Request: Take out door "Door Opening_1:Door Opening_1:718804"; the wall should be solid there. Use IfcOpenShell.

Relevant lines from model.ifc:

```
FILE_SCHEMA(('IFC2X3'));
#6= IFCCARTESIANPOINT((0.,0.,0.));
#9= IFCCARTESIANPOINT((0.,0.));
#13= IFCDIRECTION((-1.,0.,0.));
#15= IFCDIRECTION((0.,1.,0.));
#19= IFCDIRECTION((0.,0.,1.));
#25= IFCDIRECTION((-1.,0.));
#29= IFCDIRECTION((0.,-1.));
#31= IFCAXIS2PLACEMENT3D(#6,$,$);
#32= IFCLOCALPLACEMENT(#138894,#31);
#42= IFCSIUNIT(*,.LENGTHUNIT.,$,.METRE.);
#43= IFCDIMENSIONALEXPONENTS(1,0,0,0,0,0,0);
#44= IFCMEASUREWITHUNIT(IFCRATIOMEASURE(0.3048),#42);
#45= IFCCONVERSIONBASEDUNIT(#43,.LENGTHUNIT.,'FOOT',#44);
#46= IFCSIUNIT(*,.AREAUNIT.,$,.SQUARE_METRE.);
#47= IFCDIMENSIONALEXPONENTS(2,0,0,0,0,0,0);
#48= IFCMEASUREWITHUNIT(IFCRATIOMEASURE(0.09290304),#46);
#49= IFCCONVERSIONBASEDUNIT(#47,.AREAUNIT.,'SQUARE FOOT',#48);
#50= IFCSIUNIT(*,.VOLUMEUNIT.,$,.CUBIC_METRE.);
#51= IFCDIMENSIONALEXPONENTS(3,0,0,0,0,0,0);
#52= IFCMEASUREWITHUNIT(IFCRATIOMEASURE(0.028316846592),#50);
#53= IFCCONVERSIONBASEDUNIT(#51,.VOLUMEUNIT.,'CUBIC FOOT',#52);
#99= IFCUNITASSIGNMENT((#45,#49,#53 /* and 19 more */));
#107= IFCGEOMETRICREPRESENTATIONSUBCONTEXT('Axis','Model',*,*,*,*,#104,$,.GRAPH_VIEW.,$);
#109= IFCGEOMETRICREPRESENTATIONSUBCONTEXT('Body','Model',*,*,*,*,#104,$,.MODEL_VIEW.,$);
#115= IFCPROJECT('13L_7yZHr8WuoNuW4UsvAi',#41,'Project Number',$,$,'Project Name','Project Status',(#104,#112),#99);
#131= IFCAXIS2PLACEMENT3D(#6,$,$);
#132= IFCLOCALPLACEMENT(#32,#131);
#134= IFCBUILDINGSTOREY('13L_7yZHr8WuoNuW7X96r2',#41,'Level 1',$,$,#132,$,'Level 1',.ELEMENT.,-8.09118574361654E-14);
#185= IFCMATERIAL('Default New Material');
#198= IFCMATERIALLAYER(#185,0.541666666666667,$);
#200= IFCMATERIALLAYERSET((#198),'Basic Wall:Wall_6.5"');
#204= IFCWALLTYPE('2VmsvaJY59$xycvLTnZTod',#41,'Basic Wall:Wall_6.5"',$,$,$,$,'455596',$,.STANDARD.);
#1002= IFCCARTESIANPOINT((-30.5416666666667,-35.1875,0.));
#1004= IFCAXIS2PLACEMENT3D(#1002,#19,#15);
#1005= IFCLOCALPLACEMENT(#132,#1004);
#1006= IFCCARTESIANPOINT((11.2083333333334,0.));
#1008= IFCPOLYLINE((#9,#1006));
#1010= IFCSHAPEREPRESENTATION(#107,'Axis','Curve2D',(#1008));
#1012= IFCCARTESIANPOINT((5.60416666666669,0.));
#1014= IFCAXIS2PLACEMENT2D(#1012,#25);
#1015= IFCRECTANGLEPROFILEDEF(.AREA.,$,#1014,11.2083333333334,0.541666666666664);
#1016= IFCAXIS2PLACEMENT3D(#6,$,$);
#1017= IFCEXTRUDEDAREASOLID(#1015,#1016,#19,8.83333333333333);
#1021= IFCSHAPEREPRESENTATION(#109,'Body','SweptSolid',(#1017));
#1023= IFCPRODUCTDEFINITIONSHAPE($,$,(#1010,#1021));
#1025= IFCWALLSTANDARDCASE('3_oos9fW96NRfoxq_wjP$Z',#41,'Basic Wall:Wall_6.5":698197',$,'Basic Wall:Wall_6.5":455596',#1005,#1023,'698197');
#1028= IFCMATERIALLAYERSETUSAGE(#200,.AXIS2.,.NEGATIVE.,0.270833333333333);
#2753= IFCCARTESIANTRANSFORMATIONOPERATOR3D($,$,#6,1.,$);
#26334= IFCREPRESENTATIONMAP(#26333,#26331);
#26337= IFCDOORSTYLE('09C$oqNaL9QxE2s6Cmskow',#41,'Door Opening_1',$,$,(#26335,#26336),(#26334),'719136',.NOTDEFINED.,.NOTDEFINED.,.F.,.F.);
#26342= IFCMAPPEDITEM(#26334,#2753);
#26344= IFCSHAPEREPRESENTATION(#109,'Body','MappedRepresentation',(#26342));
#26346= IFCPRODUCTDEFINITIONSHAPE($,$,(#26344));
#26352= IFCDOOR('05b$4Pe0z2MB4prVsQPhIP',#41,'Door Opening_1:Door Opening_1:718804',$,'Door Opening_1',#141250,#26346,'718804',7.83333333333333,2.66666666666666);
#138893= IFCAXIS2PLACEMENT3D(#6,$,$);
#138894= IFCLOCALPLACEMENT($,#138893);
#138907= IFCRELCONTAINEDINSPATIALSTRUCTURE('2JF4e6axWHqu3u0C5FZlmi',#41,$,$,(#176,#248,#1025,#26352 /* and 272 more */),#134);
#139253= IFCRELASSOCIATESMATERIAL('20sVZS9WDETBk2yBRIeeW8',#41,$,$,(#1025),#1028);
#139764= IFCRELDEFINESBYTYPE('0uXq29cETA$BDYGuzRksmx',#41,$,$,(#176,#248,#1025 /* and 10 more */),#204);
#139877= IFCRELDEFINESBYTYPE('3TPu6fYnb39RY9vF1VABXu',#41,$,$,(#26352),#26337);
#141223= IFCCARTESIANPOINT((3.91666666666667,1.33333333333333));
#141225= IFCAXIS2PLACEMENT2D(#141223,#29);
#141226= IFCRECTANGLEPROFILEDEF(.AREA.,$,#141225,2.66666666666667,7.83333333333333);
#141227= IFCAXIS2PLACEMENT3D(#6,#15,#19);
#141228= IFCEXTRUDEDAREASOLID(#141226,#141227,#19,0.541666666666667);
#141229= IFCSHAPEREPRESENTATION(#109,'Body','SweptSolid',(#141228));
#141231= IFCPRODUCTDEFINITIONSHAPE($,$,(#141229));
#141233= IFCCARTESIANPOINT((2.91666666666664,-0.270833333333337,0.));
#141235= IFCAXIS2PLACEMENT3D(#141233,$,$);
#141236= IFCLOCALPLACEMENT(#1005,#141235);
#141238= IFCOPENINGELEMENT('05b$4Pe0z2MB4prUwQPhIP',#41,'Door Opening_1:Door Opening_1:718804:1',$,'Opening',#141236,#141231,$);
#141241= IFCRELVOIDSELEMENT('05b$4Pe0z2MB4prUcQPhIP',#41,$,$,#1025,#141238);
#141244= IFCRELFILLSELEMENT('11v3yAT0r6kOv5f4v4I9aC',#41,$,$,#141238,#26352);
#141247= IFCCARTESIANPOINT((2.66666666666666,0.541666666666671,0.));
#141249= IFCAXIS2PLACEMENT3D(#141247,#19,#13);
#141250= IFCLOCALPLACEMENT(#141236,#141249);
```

```python
import ifcopenshell
import ifcopenshell.api.feature
import ifcopenshell.api.root
import ifcopenshell.geom
import ifcopenshell.util.shape

model = ifcopenshell.open("model.ifc")
settings = ifcopenshell.geom.settings()


def volume(element):
    """Net volume in cubic metres, openings subtracted."""
    shape = ifcopenshell.geom.create_shape(settings, element)
    return ifcopenshell.util.shape.get_volume(shape.geometry)


door = model.by_guid("05b$4Pe0z2MB4prVsQPhIP")
opening = door.FillsVoids[0].RelatingOpeningElement
wall = opening.VoidsElements[0].RelatingBuildingElement
before = volume(wall)

ifcopenshell.api.root.remove_product(model, product=door)
ifcopenshell.api.feature.remove_feature(model, feature=opening)

after = volume(wall)

print(f"wall volume {before:.3f} -> {after:.3f} m3")

model.write("model_rev.ifc")
```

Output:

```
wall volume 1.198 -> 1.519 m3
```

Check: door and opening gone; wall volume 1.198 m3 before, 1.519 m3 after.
